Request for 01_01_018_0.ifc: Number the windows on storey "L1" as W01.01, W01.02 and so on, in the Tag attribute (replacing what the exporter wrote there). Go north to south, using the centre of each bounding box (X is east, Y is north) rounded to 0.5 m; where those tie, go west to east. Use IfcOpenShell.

First a look at what the model holds.

```python
import ifcopenshell
import ifcopenshell.util.element
import ifcopenshell.util.placement

model = ifcopenshell.open("01_01_018_0.ifc")
print(model.schema)
storey = next(s for s in model.by_type("IfcBuildingStorey") if s.Name == "L1")
windows = [e for e in ifcopenshell.util.element.get_decomposition(storey) if e.is_a("IfcWindow")]
for e in sorted(windows, key=lambda e: e.id()):
    origin = ifcopenshell.util.placement.get_local_placement(e.ObjectPlacement)[:3, 3]
    print(e.id(), e.Tag, e.Name, origin.round(2) + 0.0, sep=" | ")
```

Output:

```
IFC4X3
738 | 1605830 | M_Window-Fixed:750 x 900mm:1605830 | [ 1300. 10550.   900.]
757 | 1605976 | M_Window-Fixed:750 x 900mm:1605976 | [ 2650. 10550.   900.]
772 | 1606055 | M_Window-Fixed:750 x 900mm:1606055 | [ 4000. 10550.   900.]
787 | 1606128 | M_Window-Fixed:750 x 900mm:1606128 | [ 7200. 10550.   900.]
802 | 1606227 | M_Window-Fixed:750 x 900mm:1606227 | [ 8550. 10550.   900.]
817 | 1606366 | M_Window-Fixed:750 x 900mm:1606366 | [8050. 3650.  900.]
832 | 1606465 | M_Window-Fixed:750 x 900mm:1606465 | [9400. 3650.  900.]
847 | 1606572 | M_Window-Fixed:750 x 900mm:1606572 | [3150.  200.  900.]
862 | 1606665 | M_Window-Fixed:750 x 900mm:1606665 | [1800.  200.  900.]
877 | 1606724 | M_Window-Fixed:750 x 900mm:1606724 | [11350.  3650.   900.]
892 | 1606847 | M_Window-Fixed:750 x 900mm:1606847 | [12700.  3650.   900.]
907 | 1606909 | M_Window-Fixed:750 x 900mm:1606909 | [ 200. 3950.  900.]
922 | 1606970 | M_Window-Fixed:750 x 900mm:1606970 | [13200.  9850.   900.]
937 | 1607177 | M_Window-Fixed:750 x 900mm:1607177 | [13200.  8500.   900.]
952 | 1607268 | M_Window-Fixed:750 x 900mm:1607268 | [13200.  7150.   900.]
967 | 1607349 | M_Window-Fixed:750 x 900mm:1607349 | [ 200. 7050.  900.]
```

```python
import ifcopenshell
import ifcopenshell.geom
import ifcopenshell.util.element
import ifcopenshell.util.shape

model = ifcopenshell.open("01_01_018_0.ifc")
settings = ifcopenshell.geom.settings()
settings.set("use-world-coords", True)


def centre(element):
    shape = ifcopenshell.geom.create_shape(settings, element)
    return ifcopenshell.util.shape.get_bbox_centroid(shape.geometry)


storey = next(s for s in model.by_type("IfcBuildingStorey") if s.Name == "L1")
windows = [e for e in ifcopenshell.util.element.get_decomposition(storey) if e.is_a("IfcWindow")]

# Insertion points can sit at a corner or the storey origin, so sort by the geometry (in metres).
centres = {e: centre(e) for e in windows}
windows.sort(key=lambda e: (-round(centres[e][1] / 0.5), centres[e][0]))

for i, e in enumerate(windows, start=1):
    number = f"W01.{i:02d}"
    e.Tag = number
    print(e.id(), number)

model.write("01_01_018_0-out.ifc")
```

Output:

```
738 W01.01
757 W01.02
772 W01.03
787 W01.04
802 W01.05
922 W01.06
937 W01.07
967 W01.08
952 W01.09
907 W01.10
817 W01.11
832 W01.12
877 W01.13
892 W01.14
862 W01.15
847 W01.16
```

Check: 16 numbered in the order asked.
